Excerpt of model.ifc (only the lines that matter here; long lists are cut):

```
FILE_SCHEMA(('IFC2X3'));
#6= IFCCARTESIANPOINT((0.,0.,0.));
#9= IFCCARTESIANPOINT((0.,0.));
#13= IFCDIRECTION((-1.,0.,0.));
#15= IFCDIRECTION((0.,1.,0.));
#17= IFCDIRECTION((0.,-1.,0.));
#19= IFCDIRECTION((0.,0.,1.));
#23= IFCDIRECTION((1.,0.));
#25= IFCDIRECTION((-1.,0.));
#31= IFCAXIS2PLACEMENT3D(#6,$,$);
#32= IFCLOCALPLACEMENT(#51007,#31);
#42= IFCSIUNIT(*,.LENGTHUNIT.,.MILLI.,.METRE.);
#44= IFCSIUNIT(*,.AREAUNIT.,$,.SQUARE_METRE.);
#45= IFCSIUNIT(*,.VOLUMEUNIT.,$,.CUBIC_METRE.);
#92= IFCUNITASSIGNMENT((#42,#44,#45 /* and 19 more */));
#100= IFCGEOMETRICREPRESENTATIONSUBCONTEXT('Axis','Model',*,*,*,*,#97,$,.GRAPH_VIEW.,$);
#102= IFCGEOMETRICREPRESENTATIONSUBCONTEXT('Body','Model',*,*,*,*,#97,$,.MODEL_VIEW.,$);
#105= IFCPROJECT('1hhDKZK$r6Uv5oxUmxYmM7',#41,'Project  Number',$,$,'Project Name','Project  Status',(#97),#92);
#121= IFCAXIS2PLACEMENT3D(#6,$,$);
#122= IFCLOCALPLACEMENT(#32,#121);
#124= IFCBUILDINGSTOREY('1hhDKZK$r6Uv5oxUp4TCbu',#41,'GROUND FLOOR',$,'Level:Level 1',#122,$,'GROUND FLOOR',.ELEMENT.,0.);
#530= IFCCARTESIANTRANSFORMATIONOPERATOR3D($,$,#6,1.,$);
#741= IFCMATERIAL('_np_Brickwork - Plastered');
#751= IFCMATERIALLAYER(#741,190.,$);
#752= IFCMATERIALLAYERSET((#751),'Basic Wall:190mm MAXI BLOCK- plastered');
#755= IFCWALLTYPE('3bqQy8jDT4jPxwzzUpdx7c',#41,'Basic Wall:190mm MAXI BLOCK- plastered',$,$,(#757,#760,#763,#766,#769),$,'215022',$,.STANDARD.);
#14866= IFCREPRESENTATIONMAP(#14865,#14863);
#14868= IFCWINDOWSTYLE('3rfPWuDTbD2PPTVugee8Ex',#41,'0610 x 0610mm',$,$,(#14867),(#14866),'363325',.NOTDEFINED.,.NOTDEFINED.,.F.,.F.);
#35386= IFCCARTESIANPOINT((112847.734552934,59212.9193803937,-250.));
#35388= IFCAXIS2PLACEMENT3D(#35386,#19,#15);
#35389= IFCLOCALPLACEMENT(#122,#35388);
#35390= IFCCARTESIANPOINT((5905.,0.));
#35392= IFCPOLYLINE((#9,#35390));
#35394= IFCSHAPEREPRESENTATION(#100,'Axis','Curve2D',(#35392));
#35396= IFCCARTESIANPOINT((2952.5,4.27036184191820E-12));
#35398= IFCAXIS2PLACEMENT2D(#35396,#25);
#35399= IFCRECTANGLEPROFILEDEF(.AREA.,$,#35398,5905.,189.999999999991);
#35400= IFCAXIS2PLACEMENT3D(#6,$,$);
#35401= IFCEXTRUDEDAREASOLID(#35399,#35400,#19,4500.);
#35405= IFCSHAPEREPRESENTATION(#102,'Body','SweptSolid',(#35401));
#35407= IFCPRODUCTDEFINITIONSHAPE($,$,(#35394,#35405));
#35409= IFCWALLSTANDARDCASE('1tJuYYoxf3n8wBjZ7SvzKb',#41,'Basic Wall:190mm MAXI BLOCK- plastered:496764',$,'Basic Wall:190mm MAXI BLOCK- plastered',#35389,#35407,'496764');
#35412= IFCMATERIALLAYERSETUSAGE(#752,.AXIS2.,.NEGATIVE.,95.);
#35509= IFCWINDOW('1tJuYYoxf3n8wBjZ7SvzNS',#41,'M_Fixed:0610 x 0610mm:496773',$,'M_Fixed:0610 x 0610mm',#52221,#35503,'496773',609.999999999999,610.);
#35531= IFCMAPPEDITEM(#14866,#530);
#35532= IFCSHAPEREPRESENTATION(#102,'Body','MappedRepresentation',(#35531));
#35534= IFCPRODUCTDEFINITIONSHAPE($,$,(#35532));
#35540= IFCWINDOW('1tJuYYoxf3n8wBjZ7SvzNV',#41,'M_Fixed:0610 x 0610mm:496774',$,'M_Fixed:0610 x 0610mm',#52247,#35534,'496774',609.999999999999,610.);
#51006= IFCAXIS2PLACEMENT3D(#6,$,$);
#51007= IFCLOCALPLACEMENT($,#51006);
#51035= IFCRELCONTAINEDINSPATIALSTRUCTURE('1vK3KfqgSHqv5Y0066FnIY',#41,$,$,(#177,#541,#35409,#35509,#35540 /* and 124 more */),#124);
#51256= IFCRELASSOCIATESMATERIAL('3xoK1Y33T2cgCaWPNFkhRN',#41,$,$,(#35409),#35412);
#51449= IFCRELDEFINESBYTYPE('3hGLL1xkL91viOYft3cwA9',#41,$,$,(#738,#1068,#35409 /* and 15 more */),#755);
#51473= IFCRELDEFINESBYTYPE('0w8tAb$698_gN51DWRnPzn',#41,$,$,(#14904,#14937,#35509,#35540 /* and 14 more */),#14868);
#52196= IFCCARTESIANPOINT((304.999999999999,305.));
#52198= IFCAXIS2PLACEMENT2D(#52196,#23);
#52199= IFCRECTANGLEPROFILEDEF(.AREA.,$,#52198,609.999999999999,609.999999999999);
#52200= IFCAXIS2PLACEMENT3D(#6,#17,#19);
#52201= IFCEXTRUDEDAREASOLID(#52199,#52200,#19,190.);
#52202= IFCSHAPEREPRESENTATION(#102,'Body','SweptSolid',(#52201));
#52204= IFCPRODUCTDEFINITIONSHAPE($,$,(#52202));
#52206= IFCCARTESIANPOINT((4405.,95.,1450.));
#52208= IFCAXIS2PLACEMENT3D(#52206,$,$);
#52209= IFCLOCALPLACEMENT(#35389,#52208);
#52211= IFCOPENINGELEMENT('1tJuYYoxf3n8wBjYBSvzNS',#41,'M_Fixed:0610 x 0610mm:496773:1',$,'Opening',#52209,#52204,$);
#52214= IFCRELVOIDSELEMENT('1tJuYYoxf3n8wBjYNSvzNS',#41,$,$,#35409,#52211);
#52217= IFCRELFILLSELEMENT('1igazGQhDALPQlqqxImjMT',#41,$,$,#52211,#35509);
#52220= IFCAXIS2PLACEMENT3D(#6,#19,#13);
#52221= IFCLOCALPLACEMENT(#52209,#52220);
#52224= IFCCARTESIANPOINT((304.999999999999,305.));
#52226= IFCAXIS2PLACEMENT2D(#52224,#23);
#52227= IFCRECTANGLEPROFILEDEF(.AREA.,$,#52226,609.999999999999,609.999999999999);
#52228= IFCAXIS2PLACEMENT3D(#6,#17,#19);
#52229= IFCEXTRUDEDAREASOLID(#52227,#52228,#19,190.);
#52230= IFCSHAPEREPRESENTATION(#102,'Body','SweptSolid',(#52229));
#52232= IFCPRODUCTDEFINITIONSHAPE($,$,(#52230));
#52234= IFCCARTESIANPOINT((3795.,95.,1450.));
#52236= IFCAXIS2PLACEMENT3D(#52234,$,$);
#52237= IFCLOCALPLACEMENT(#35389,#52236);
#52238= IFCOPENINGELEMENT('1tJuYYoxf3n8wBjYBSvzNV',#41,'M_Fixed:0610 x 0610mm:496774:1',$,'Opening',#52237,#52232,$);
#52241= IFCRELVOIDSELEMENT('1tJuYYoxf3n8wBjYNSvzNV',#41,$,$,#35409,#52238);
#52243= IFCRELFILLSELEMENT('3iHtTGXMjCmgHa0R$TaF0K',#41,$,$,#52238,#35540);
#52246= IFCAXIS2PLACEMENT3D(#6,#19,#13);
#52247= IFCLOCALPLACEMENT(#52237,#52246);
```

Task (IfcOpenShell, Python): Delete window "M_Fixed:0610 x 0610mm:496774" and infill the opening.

```python
import ifcopenshell
import ifcopenshell.api.feature
import ifcopenshell.api.root
import ifcopenshell.geom
import ifcopenshell.util.shape

model = ifcopenshell.open("model.ifc")
settings = ifcopenshell.geom.settings()


def volume(element):
    """Net volume in cubic metres, openings subtracted."""
    shape = ifcopenshell.geom.create_shape(settings, element)
    return ifcopenshell.util.shape.get_volume(shape.geometry)


window = model.by_guid("1tJuYYoxf3n8wBjZ7SvzNV")
opening = window.FillsVoids[0].RelatingOpeningElement
wall = opening.VoidsElements[0].RelatingBuildingElement
before = volume(wall)

ifcopenshell.api.root.remove_product(model, product=window)
ifcopenshell.api.feature.remove_feature(model, feature=opening)

after = volume(wall)

print(f"wall volume {before:.3f} -> {after:.3f} m3")

model.write("model_updated.ifc")
```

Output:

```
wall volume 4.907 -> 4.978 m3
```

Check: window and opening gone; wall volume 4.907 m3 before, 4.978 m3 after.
